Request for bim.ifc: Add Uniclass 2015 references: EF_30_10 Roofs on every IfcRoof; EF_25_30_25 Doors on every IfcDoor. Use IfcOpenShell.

First a look at what the model holds.

```python
import ifcopenshell

model = ifcopenshell.open("bim.ifc")
print(model.schema)
print("classifications:", [c.Name for c in model.by_type("IfcClassification")])
for ifc_class in ("IfcDoor", "IfcRoof", "IfcStair", "IfcWall", "IfcWindow"):
    print(ifc_class, len(model.by_type(ifc_class)))
```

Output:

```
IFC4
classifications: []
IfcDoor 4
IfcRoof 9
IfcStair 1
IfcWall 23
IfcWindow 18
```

```python
import ifcopenshell
import ifcopenshell.api.classification

model = ifcopenshell.open("bim.ifc")

system = ifcopenshell.api.classification.add_classification(model, classification="Uniclass 2015")

codes = {
    "IfcRoof": ("EF_30_10", "Roofs"),
    "IfcDoor": ("EF_25_30_25", "Doors"),
}
for ifc_class, (code, name) in codes.items():
    products = model.by_type(ifc_class)
    ifcopenshell.api.classification.add_reference(
        model, products=products, classification=system, identification=code, name=name
    )
    print(code, len(products))

model.write("bim_v2.ifc")
```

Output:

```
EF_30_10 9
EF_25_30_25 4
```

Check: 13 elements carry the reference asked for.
